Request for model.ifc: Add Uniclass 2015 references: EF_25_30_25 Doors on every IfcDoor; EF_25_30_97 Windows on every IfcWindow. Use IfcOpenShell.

First a look at what the model holds.

```python
import ifcopenshell

model = ifcopenshell.open("model.ifc")
print(model.schema)
print("classifications:", [c.Name for c in model.by_type("IfcClassification")])
for ifc_class in ("IfcDoor", "IfcRoof", "IfcStair", "IfcWall", "IfcWindow"):
    print(ifc_class, len(model.by_type(ifc_class)))
```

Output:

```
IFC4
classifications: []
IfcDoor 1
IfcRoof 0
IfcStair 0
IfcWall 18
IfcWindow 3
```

```python
import ifcopenshell
import ifcopenshell.api.classification

model = ifcopenshell.open("model.ifc")

system = ifcopenshell.api.classification.add_classification(model, classification="Uniclass 2015")

codes = {
    "IfcDoor": ("EF_25_30_25", "Doors"),
    "IfcWindow": ("EF_25_30_97", "Windows"),
}
for ifc_class, (code, name) in codes.items():
    products = model.by_type(ifc_class)
    ifcopenshell.api.classification.add_reference(
        model, products=products, classification=system, identification=code, name=name
    )
    print(code, len(products))

model.write("model_v2.ifc")
```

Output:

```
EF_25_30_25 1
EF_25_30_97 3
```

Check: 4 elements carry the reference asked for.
